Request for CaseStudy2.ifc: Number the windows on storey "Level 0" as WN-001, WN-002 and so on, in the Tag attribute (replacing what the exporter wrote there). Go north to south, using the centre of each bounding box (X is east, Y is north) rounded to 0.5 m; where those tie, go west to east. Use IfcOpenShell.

First a look at what the model holds.

```python
import ifcopenshell
import ifcopenshell.util.element
import ifcopenshell.util.placement

model = ifcopenshell.open("CaseStudy2.ifc")
print(model.schema)
storey = next(s for s in model.by_type("IfcBuildingStorey") if s.Name == "Level 0")
windows = [e for e in ifcopenshell.util.element.get_decomposition(storey) if e.is_a("IfcWindow")]
for e in sorted(windows, key=lambda e: e.id()):
    origin = ifcopenshell.util.placement.get_local_placement(e.ObjectPlacement)[:3, 3]
    print(e.id(), e.Tag, e.Name, origin.round(2) + 0.0, sep=" | ")
```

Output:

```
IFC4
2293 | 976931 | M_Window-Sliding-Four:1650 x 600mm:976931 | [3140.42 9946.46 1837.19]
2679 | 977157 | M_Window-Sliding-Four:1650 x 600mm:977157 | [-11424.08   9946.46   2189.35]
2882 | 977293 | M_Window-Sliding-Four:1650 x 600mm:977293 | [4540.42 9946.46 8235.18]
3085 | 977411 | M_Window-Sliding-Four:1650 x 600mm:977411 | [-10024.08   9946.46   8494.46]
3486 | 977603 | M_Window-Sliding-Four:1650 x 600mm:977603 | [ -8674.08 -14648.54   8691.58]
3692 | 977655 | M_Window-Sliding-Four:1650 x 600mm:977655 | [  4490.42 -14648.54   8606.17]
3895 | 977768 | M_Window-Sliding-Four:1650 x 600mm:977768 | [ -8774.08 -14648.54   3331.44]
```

```python
import ifcopenshell
import ifcopenshell.geom
import ifcopenshell.util.element
import ifcopenshell.util.shape

model = ifcopenshell.open("CaseStudy2.ifc")
settings = ifcopenshell.geom.settings()
settings.set("use-world-coords", True)


def centre(element):
    shape = ifcopenshell.geom.create_shape(settings, element)
    return ifcopenshell.util.shape.get_bbox_centroid(shape.geometry)


storey = next(s for s in model.by_type("IfcBuildingStorey") if s.Name == "Level 0")
windows = [e for e in ifcopenshell.util.element.get_decomposition(storey) if e.is_a("IfcWindow")]

# Insertion points can sit at a corner or the storey origin, so sort by the geometry (in metres).
centres = {e: centre(e) for e in windows}
windows.sort(key=lambda e: (-round(centres[e][1] / 0.5), centres[e][0]))

for i, e in enumerate(windows, start=1):
    number = f"WN-0{i:02d}"
    e.Tag = number
    print(e.id(), number)

model.write("CaseStudy2_updated.ifc")
```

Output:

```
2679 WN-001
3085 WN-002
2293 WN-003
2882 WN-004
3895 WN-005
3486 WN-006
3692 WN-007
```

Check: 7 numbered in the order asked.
